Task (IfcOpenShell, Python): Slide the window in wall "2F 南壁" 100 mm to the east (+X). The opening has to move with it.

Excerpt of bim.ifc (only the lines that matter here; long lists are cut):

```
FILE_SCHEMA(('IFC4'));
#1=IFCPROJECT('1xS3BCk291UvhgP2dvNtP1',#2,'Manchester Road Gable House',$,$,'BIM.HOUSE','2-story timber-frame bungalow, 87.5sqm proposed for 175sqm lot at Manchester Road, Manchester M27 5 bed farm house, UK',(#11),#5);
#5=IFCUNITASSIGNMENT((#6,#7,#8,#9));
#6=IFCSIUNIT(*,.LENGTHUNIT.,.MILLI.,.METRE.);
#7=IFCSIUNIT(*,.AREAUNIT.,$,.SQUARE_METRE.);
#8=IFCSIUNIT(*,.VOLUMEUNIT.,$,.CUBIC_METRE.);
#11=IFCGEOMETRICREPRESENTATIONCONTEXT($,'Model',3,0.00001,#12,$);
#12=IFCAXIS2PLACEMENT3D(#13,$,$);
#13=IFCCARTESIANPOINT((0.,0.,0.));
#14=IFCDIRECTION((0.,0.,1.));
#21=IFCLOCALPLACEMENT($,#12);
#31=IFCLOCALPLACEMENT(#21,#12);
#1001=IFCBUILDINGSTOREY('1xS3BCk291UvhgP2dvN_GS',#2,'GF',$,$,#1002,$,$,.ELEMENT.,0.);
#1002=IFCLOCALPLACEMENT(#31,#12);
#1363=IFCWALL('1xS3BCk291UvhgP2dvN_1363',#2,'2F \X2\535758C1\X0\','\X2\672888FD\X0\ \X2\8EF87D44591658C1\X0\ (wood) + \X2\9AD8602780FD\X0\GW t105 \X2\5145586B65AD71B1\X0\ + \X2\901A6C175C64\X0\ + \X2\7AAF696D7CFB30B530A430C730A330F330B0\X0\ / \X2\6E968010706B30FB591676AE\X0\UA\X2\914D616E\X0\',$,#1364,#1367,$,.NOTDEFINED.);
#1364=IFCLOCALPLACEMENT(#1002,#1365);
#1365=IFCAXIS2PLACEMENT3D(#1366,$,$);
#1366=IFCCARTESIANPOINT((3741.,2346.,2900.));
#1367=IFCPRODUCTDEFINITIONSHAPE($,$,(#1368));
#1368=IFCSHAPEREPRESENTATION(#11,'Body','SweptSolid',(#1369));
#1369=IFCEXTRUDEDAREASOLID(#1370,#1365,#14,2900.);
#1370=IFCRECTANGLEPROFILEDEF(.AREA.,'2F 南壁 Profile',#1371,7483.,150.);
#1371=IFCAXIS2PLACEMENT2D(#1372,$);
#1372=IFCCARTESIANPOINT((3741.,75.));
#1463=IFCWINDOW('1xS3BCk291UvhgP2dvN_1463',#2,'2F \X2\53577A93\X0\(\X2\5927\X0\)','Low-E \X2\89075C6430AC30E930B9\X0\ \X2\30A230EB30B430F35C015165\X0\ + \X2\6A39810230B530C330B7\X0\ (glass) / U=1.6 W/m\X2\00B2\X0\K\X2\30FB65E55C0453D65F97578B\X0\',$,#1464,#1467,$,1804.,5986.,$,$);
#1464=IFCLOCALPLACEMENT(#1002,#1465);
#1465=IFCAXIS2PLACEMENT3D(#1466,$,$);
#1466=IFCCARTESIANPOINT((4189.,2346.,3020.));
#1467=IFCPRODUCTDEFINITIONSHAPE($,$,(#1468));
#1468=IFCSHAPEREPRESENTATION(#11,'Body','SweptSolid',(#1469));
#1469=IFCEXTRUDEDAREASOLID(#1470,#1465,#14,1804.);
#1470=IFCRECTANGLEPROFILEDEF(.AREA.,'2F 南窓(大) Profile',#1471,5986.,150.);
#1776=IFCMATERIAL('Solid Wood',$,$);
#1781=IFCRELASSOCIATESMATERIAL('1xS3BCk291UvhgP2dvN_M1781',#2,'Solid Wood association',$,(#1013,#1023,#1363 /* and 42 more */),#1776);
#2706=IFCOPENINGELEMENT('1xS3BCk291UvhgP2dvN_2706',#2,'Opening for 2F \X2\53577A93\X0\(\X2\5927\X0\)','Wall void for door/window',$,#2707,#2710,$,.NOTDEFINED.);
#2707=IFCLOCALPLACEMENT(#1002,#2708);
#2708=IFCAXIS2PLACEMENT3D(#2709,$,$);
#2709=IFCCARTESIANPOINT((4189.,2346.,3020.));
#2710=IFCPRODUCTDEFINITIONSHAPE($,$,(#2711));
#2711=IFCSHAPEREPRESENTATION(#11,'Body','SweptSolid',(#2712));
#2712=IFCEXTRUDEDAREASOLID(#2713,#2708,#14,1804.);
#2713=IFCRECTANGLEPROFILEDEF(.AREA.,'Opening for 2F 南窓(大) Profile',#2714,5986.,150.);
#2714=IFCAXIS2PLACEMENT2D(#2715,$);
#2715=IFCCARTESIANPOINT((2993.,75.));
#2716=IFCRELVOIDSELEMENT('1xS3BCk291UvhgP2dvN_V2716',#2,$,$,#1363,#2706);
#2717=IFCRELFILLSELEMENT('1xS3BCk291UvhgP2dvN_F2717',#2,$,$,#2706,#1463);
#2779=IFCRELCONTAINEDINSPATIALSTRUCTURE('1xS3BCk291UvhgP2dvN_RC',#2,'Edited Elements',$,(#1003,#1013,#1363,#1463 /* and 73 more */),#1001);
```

```python
import ifcopenshell
import ifcopenshell.api.geometry
import ifcopenshell.util.placement

model = ifcopenshell.open("bim.ifc")

window = model.by_guid("1xS3BCk291UvhgP2dvN_1463")
opening = window.FillsVoids[0].RelatingOpeningElement
wall = opening.VoidsElements[0].RelatingBuildingElement

wall_matrix = ifcopenshell.util.placement.get_local_placement(wall.ObjectPlacement)
shift = wall_matrix[:3, 0] * 100.0
before = ifcopenshell.util.placement.get_local_placement(window.ObjectPlacement)[:3, 3].copy()

# The window is not placed relative to its opening, so move both.
for product in (opening, window):
    matrix = ifcopenshell.util.placement.get_local_placement(product.ObjectPlacement)
    matrix[:3, 3] += shift
    ifcopenshell.api.geometry.edit_object_placement(model, product=product, matrix=matrix, is_si=False)

after = ifcopenshell.util.placement.get_local_placement(window.ObjectPlacement)[:3, 3]
print("window moved by", (after - before).round(3) + 0.0)

model.write("bim_updated.ifc")
```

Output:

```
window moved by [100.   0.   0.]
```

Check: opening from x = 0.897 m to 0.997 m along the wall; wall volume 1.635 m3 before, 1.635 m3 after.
